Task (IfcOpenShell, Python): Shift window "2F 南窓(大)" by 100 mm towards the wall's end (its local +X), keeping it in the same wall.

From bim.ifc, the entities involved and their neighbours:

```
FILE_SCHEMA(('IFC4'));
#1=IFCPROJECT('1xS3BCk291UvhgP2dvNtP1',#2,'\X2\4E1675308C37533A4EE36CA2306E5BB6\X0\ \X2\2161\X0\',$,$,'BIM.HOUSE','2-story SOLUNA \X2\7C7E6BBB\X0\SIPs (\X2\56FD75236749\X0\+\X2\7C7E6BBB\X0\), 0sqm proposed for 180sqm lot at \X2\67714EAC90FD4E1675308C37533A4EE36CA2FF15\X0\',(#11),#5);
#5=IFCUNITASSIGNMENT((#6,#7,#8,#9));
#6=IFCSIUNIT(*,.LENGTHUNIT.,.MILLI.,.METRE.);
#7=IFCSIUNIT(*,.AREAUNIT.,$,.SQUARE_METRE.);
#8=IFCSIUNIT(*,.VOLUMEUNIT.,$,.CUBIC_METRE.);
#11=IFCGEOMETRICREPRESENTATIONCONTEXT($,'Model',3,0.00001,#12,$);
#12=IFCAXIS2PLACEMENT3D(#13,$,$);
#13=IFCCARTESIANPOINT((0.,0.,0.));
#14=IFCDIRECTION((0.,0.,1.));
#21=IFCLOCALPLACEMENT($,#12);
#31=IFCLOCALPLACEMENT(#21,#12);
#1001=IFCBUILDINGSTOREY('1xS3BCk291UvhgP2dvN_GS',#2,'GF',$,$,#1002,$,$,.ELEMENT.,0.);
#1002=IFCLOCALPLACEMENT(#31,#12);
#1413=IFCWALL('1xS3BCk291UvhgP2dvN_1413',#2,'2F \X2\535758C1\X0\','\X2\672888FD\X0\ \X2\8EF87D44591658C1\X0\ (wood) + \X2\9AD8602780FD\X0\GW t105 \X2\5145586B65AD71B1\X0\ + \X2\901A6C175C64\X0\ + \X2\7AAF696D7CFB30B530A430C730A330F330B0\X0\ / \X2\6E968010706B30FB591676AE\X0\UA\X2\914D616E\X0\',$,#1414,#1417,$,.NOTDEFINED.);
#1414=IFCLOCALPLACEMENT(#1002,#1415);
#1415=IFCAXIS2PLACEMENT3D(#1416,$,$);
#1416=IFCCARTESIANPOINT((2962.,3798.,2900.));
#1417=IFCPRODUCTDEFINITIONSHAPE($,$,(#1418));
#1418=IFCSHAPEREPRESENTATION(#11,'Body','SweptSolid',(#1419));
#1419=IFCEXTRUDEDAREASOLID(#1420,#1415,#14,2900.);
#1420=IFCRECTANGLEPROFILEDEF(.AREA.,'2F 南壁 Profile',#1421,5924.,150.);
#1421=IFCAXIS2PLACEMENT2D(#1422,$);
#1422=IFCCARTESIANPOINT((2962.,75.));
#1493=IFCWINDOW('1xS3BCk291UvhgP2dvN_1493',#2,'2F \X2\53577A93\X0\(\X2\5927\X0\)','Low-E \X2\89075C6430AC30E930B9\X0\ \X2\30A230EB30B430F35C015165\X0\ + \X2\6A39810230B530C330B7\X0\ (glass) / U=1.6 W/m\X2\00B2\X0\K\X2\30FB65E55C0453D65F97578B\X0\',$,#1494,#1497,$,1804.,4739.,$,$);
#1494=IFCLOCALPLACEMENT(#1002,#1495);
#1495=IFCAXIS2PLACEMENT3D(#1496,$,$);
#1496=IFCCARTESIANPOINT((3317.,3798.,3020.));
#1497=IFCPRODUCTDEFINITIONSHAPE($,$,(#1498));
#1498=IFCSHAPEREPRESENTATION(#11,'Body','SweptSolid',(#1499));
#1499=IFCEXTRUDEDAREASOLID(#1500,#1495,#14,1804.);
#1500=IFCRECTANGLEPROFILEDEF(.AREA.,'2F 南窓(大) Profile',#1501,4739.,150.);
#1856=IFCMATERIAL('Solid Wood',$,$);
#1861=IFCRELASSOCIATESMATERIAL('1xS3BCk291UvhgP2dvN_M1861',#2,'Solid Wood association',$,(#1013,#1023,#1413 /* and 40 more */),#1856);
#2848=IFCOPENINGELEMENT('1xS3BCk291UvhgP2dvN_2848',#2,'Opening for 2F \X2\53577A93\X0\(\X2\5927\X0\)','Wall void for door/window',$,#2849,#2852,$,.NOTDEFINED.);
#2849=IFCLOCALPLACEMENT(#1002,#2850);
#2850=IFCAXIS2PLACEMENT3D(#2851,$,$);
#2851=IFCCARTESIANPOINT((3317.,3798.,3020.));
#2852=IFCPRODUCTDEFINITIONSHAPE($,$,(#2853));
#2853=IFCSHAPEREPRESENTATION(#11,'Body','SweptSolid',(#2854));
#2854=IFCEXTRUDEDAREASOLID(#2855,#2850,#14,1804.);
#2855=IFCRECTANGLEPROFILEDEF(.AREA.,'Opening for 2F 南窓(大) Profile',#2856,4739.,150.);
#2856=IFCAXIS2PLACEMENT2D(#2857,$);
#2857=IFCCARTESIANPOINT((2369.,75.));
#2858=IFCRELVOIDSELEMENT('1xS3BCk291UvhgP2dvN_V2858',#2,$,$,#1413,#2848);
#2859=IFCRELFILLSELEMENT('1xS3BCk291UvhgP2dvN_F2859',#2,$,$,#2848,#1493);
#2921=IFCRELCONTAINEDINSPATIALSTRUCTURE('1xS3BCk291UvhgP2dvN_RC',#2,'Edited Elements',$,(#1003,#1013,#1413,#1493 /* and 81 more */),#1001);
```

```python
import ifcopenshell
import ifcopenshell.api.geometry
import ifcopenshell.util.placement

model = ifcopenshell.open("bim.ifc")

window = model.by_guid("1xS3BCk291UvhgP2dvN_1493")
opening = window.FillsVoids[0].RelatingOpeningElement
wall = opening.VoidsElements[0].RelatingBuildingElement

wall_matrix = ifcopenshell.util.placement.get_local_placement(wall.ObjectPlacement)
shift = wall_matrix[:3, 0] * 100.0
before = ifcopenshell.util.placement.get_local_placement(window.ObjectPlacement)[:3, 3].copy()

# The window is not placed relative to its opening, so move both.
for product in (opening, window):
    matrix = ifcopenshell.util.placement.get_local_placement(product.ObjectPlacement)
    matrix[:3, 3] += shift
    ifcopenshell.api.geometry.edit_object_placement(model, product=product, matrix=matrix, is_si=False)

after = ifcopenshell.util.placement.get_local_placement(window.ObjectPlacement)[:3, 3]
print("window moved by", (after - before).round(3) + 0.0)

model.write("bim_edited.ifc")
```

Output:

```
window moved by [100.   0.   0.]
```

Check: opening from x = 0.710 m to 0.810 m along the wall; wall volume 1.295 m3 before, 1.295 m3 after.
